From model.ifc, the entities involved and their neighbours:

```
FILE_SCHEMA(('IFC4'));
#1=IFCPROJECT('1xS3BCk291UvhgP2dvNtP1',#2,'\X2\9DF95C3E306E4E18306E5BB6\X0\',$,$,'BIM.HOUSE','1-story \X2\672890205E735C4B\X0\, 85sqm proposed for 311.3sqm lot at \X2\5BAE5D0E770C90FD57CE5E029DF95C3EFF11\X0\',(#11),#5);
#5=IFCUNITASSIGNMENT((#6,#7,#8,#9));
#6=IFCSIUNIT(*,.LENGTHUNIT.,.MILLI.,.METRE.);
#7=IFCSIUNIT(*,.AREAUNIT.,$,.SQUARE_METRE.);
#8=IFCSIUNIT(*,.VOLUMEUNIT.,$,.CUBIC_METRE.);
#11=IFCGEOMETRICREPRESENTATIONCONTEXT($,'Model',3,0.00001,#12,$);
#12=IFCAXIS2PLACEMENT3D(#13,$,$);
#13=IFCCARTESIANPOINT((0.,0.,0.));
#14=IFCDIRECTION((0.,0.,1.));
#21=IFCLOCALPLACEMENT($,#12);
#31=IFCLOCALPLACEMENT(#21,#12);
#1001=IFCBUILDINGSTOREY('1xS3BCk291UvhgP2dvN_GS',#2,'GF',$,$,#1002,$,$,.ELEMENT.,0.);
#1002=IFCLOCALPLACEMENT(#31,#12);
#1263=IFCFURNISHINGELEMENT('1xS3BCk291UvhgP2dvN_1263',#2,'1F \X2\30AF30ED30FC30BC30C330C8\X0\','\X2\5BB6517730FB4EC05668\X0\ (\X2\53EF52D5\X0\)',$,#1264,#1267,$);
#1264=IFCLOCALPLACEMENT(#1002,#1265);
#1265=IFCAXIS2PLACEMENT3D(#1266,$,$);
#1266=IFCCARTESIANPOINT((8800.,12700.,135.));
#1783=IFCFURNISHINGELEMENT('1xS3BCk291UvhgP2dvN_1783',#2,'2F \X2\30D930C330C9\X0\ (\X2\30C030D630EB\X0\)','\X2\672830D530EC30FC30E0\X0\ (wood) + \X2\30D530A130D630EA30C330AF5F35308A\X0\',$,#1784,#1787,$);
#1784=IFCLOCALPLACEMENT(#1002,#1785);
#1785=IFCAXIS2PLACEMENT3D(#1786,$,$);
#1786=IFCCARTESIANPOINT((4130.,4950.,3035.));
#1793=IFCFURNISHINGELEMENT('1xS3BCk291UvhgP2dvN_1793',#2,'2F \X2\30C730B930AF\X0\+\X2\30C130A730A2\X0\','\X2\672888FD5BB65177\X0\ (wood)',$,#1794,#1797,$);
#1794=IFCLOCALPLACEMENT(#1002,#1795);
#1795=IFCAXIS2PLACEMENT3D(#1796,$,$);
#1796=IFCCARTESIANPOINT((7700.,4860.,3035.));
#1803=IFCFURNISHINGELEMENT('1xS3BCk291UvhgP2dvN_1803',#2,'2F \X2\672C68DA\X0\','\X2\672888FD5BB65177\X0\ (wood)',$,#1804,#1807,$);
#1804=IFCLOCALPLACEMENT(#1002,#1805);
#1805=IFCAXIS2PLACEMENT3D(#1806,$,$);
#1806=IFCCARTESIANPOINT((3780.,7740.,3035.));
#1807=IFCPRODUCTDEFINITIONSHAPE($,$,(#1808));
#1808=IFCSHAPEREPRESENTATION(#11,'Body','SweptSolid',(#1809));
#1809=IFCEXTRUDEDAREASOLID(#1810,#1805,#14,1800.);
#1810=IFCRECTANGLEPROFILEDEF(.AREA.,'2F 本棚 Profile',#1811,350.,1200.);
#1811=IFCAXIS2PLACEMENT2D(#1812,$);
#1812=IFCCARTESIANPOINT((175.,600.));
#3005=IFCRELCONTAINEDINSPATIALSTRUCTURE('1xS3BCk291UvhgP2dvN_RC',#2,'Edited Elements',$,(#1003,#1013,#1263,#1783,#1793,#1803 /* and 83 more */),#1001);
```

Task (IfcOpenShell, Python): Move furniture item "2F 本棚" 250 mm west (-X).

```python
import ifcopenshell
import ifcopenshell.api.geometry
import ifcopenshell.util.placement

model = ifcopenshell.open("model.ifc")

item = model.by_guid("1xS3BCk291UvhgP2dvN_1803")
matrix = ifcopenshell.util.placement.get_local_placement(item.ObjectPlacement)
matrix[0, 3] -= 250.0
ifcopenshell.api.geometry.edit_object_placement(model, product=item, matrix=matrix, is_si=False)

print(ifcopenshell.util.placement.get_local_placement(item.ObjectPlacement).round(3) + 0.0)

model.write("model_edited.ifc")
```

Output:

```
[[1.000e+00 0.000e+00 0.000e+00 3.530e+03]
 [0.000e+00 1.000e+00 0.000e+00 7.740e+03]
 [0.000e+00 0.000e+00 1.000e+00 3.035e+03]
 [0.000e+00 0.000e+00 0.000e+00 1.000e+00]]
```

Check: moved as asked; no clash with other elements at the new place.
